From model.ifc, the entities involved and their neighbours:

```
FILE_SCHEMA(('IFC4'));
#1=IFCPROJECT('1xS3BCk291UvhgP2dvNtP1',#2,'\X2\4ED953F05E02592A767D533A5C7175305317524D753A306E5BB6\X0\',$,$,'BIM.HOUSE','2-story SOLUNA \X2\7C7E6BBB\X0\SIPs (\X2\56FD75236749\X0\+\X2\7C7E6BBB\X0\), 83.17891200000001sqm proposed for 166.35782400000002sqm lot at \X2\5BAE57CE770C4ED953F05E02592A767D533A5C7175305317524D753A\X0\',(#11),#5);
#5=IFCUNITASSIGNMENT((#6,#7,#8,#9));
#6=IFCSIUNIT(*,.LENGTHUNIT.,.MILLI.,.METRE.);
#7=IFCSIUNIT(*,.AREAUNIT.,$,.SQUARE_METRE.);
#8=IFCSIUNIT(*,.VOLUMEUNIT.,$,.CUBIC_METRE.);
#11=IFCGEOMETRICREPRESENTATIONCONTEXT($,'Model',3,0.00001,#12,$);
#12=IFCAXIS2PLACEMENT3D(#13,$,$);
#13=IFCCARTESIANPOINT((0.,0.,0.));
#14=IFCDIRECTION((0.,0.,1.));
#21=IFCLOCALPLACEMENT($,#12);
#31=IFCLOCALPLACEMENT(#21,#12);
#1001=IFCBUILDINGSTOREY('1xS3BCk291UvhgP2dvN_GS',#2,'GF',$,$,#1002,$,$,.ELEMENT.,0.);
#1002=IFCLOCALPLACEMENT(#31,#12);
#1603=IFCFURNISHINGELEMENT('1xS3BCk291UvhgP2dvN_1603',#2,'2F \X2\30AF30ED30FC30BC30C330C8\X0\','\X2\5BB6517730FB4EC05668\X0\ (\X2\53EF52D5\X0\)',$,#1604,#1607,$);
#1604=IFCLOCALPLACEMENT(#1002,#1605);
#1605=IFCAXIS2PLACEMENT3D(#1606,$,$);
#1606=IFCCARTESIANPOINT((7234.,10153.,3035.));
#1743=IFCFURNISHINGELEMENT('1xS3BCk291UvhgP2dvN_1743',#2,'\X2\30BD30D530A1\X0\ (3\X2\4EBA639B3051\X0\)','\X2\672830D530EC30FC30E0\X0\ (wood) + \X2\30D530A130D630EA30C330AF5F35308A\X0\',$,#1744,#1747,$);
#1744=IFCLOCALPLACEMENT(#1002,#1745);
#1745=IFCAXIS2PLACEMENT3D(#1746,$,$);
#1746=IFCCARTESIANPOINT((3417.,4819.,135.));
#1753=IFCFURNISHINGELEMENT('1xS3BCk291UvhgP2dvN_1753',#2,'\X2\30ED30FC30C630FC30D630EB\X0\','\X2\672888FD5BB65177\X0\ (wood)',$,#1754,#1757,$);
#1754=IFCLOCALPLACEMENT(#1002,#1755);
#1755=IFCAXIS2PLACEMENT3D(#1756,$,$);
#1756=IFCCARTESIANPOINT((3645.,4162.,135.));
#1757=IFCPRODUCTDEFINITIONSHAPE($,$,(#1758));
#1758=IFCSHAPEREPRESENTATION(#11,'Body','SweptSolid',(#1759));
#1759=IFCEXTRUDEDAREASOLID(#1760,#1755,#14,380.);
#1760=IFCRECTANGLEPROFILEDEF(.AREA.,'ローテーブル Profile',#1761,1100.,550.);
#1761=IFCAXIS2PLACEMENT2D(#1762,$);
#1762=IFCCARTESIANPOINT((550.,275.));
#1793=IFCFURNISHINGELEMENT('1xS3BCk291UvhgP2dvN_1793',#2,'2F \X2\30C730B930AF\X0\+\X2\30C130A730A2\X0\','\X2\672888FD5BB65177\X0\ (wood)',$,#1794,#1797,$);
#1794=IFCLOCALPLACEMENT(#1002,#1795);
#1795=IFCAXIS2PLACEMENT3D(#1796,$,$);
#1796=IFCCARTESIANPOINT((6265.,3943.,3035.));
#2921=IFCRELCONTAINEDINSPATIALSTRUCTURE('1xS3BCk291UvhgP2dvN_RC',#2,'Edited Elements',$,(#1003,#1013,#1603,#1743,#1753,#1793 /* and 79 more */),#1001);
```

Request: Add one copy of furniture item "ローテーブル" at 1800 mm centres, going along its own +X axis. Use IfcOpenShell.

```python
import ifcopenshell
import ifcopenshell.api.geometry
import ifcopenshell.api.root
import ifcopenshell.util.element
import ifcopenshell.util.placement
import ifcopenshell.util.unit

model = ifcopenshell.open("model.ifc")
unit_scale = ifcopenshell.util.unit.calculate_unit_scale(model)


def reuse_history(source, copy):
    """copy_class also copies each property set's owner history, people and application; keep the originals."""
    for rel in copy.IsDefinedBy:
        if rel.is_a("IfcRelDefinesByProperties") and (history := rel.RelatingPropertyDefinition.OwnerHistory):
            rel.RelatingPropertyDefinition.OwnerHistory = source.OwnerHistory
            ifcopenshell.util.element.remove_deep2(model, history)


source = model.by_guid("1xS3BCk291UvhgP2dvN_1753")
base = ifcopenshell.util.placement.get_local_placement(source.ObjectPlacement)
step = base[:3, 0] * 1.8 / unit_scale

for i in range(1, 2):
    copy = ifcopenshell.api.root.copy_class(model, product=source)
    copy.Representation = ifcopenshell.util.element.copy_deep(
        model, source.Representation, exclude=["IfcGeometricRepresentationContext", "IfcRepresentationMap"]
    )
    reuse_history(source, copy)
    matrix = base.copy()
    matrix[:3, 3] += i * step
    print("added at", matrix[:3, 3].round(3) + 0.0)
    ifcopenshell.api.geometry.edit_object_placement(model, product=copy, matrix=matrix, is_si=False)

model.write("model_edited.ifc")
```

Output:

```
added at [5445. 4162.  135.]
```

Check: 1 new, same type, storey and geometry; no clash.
